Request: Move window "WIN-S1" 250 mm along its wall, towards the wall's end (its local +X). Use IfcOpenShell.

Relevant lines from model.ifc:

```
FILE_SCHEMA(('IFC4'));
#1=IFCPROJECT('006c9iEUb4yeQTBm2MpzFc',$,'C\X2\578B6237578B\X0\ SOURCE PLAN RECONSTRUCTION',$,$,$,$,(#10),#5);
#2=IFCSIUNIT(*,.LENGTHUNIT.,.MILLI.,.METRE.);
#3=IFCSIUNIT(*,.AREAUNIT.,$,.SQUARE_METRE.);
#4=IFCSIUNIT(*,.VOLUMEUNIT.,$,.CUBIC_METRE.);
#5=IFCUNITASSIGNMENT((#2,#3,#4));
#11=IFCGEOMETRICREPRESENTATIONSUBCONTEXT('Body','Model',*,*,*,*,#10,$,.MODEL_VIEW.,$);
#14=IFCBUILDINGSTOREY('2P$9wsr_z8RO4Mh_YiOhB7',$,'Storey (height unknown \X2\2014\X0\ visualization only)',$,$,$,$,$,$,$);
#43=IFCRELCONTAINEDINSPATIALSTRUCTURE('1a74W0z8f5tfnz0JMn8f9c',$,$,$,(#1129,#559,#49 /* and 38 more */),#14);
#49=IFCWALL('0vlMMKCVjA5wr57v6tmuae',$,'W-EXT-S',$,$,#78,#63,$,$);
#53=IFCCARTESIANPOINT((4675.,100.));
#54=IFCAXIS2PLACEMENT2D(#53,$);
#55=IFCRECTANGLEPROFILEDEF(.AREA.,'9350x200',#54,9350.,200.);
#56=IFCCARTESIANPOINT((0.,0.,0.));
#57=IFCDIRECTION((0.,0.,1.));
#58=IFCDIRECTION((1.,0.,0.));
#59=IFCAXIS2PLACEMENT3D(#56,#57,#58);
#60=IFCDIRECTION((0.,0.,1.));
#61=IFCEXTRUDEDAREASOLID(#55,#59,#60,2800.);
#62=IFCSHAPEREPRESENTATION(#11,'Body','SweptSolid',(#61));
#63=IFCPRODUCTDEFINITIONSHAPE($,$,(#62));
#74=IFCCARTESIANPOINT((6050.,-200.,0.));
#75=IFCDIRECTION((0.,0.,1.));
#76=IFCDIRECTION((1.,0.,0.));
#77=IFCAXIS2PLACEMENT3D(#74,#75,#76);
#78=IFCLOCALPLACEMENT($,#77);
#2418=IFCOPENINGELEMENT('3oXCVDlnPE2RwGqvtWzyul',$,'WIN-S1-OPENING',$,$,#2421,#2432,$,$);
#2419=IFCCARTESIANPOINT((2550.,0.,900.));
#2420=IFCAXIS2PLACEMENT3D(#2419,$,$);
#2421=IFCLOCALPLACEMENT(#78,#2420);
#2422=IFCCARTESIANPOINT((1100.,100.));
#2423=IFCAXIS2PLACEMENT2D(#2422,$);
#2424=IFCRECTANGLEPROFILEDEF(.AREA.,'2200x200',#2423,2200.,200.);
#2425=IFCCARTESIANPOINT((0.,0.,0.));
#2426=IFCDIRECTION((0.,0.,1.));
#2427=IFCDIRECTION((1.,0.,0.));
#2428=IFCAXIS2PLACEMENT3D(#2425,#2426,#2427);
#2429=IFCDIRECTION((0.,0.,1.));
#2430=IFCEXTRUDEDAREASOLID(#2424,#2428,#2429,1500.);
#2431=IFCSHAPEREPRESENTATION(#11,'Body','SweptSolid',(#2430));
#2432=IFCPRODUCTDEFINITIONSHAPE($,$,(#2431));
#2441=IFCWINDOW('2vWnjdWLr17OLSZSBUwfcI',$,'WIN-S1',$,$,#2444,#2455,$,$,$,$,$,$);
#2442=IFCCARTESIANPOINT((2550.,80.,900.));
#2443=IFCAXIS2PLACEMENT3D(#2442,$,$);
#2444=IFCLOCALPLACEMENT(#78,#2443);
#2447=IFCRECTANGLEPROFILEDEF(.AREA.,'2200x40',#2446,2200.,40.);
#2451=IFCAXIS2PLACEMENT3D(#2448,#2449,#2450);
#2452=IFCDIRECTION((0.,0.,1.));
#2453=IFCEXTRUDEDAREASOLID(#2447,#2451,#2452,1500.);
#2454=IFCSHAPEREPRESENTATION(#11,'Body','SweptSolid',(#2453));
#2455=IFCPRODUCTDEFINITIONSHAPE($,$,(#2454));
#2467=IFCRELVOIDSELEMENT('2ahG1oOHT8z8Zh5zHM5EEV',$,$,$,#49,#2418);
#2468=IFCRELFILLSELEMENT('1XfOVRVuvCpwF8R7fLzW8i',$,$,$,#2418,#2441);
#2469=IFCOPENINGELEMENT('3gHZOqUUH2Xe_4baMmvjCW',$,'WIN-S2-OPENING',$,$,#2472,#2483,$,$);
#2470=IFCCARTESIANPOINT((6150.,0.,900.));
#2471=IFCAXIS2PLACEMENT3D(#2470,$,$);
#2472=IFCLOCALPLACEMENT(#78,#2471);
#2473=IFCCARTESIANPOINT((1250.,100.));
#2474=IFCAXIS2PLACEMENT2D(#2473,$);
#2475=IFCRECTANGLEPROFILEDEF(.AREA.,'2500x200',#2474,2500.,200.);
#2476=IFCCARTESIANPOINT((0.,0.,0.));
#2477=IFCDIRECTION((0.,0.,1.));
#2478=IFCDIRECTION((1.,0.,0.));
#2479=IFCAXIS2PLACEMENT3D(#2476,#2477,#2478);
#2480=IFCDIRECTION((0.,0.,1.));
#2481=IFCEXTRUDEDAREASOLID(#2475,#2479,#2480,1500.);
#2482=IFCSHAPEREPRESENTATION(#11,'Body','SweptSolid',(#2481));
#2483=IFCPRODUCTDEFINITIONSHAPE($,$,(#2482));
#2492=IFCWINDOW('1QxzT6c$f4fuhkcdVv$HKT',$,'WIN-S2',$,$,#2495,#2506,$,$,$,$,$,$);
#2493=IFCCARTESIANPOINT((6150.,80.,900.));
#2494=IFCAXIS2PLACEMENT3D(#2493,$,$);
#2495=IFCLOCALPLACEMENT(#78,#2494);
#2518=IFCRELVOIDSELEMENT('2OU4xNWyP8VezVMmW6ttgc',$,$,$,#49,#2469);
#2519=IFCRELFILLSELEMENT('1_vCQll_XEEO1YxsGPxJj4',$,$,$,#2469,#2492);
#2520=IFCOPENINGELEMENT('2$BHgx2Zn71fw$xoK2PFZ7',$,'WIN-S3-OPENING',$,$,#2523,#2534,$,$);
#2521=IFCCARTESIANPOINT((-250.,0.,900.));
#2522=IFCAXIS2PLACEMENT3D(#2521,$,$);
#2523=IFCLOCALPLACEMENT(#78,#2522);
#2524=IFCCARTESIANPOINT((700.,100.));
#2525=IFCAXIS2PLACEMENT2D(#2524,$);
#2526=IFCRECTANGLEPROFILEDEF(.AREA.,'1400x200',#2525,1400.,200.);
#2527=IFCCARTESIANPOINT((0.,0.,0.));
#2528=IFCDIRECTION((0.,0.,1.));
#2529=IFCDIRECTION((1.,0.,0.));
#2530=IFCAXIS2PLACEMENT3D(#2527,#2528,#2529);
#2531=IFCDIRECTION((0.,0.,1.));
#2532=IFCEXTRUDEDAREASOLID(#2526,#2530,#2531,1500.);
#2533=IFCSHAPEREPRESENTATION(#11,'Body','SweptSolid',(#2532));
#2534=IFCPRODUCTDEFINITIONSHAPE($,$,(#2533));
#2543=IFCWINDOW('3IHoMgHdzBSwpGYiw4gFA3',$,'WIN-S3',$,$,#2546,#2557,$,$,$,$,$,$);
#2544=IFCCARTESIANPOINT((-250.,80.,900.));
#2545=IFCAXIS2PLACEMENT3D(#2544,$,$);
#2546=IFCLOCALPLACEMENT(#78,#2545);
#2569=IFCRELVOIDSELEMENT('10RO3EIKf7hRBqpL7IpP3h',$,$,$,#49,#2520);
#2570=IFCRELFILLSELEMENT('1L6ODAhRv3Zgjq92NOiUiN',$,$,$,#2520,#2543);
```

```python
import ifcopenshell
import ifcopenshell.api.geometry
import ifcopenshell.util.placement
import ifcopenshell.util.unit

model = ifcopenshell.open("model.ifc")
unit_scale = ifcopenshell.util.unit.calculate_unit_scale(model)

window = model.by_id(2441)
opening = window.FillsVoids[0].RelatingOpeningElement
wall = opening.VoidsElements[0].RelatingBuildingElement

wall_matrix = ifcopenshell.util.placement.get_local_placement(wall.ObjectPlacement)
shift = wall_matrix[:3, 0] * 0.25 / unit_scale
before = ifcopenshell.util.placement.get_local_placement(window.ObjectPlacement)[:3, 3].copy()

# The window is not placed relative to its opening, so move both.
for product in (opening, window):
    matrix = ifcopenshell.util.placement.get_local_placement(product.ObjectPlacement)
    matrix[:3, 3] += shift
    ifcopenshell.api.geometry.edit_object_placement(model, product=product, matrix=matrix, is_si=False)

after = ifcopenshell.util.placement.get_local_placement(window.ObjectPlacement)[:3, 3]
print("window moved by", (after - before).round(3) + 0.0)

model.write("model_rev.ifc")
```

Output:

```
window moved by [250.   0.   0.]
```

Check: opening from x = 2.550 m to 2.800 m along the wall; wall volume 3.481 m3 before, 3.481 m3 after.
